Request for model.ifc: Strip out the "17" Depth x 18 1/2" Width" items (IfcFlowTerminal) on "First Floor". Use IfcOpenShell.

First a look at what the model holds.

```python
import ifcopenshell
import ifcopenshell.util.element

model = ifcopenshell.open("model.ifc")
print(model.schema)
storey = next(s for s in model.by_type("IfcBuildingStorey") if s.Name == "First Floor")
terminals = [e for e in ifcopenshell.util.element.get_decomposition(storey) if e.is_a("IfcFlowTerminal")]
seen = {}
for e in terminals:
    element_type = ifcopenshell.util.element.get_type(e)
    name = element_type.Name if element_type not in (None, e) else None
    seen[name] = seen.get(name, 0) + 1
for name, count in sorted(seen.items(), key=str):
    print(count, "x", name)
```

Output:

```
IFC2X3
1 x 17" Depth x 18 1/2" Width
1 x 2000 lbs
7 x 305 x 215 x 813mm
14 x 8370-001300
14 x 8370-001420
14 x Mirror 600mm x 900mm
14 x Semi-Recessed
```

```python
import ifcopenshell
import ifcopenshell.api.root
import ifcopenshell.util.element

model = ifcopenshell.open("model.ifc")

storey = next(s for s in model.by_type("IfcBuildingStorey") if s.Name == "First Floor")
terminals = [e for e in ifcopenshell.util.element.get_decomposition(storey) if e.is_a("IfcFlowTerminal")]
targets = [e for e in terminals if (t := ifcopenshell.util.element.get_type(e)) not in (None, e) and t.Name == '17" Depth x 18 1/2" Width']

for e in targets:
    ifcopenshell.api.root.remove_product(model, product=e)
print(len(targets), "removed")

model.write("model_v2.ifc")
```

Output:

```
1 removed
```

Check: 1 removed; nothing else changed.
